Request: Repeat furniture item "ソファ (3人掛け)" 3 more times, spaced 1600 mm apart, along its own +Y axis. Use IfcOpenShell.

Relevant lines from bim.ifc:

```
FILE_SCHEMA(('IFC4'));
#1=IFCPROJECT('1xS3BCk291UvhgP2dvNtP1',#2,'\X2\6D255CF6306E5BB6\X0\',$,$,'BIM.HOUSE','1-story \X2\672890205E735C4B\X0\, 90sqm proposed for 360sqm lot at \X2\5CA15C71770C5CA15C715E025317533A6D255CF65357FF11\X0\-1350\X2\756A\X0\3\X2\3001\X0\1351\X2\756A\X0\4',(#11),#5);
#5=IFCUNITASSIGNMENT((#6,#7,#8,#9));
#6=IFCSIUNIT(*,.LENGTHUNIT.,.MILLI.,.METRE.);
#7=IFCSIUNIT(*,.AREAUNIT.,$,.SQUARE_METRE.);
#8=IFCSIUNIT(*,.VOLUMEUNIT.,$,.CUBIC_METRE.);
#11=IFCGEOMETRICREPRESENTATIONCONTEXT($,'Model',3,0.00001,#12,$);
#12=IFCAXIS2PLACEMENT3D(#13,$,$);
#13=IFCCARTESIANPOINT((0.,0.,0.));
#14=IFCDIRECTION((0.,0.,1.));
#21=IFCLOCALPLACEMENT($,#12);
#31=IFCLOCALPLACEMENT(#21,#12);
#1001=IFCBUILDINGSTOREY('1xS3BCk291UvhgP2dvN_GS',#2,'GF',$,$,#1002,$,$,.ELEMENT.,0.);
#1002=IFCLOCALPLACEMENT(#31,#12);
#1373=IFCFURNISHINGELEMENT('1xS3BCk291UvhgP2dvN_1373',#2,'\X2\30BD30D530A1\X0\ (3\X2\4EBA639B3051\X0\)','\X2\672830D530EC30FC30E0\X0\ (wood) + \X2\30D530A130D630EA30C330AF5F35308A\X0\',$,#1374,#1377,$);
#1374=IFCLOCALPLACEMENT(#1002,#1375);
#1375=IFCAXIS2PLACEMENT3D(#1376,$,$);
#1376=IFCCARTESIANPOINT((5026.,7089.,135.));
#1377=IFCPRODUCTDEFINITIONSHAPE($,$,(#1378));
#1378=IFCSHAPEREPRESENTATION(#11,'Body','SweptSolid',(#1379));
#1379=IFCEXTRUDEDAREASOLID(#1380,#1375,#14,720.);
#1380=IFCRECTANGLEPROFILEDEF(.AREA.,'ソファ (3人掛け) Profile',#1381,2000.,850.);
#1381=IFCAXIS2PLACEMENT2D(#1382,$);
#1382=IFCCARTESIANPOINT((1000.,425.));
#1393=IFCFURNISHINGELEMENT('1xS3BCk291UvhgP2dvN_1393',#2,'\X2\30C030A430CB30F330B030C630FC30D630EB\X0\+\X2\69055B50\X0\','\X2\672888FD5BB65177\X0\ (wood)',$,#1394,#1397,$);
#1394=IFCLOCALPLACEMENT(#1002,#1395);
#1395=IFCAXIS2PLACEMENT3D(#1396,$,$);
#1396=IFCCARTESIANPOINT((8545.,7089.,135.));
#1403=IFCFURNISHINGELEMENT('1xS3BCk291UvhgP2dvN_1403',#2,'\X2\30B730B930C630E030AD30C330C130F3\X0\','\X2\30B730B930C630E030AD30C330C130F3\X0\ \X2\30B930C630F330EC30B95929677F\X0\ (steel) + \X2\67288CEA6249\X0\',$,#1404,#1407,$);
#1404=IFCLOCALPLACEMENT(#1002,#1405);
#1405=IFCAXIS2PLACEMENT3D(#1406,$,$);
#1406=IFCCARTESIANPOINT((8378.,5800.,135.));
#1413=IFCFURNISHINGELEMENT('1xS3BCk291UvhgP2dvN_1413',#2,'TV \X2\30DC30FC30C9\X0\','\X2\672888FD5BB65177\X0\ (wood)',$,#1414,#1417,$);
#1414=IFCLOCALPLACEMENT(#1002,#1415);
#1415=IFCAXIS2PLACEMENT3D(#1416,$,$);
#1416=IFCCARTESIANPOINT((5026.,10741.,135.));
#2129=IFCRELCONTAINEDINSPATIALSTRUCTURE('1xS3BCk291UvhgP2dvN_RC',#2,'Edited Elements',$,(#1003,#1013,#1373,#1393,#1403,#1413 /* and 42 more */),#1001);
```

```python
import ifcopenshell
import ifcopenshell.api.geometry
import ifcopenshell.api.root
import ifcopenshell.util.element
import ifcopenshell.util.placement
import ifcopenshell.util.unit

model = ifcopenshell.open("bim.ifc")
unit_scale = ifcopenshell.util.unit.calculate_unit_scale(model)


def reuse_history(source, copy):
    """copy_class also copies each property set's owner history, people and application; keep the originals."""
    for rel in copy.IsDefinedBy:
        if rel.is_a("IfcRelDefinesByProperties") and (history := rel.RelatingPropertyDefinition.OwnerHistory):
            rel.RelatingPropertyDefinition.OwnerHistory = source.OwnerHistory
            ifcopenshell.util.element.remove_deep2(model, history)


source = model.by_guid("1xS3BCk291UvhgP2dvN_1373")
base = ifcopenshell.util.placement.get_local_placement(source.ObjectPlacement)
step = base[:3, 1] * 1.6 / unit_scale

for i in range(1, 4):
    copy = ifcopenshell.api.root.copy_class(model, product=source)
    copy.Representation = ifcopenshell.util.element.copy_deep(
        model, source.Representation, exclude=["IfcGeometricRepresentationContext", "IfcRepresentationMap"]
    )
    reuse_history(source, copy)
    matrix = base.copy()
    matrix[:3, 3] += i * step
    print("added at", matrix[:3, 3].round(3) + 0.0)
    ifcopenshell.api.geometry.edit_object_placement(model, product=copy, matrix=matrix, is_si=False)

model.write("bim_updated.ifc")
```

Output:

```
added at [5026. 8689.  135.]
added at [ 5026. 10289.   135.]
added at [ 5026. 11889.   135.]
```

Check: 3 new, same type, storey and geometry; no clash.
